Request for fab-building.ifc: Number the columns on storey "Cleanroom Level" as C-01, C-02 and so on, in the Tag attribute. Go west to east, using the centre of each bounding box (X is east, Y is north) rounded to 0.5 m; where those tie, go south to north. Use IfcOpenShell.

First a look at what the model holds.

```python
import ifcopenshell
import ifcopenshell.util.element
import ifcopenshell.util.placement

model = ifcopenshell.open("fab-building.ifc")
print(model.schema)
storey = next(s for s in model.by_type("IfcBuildingStorey") if s.Name == "Cleanroom Level")
columns = [e for e in ifcopenshell.util.element.get_decomposition(storey) if e.is_a("IfcColumn")]
for e in sorted(columns, key=lambda e: e.id()):
    origin = ifcopenshell.util.placement.get_local_placement(e.ObjectPlacement)[:3, 3]
    print(e.id(), e.Tag, e.Name, origin.round(2) + 0.0, sep=" | ")
```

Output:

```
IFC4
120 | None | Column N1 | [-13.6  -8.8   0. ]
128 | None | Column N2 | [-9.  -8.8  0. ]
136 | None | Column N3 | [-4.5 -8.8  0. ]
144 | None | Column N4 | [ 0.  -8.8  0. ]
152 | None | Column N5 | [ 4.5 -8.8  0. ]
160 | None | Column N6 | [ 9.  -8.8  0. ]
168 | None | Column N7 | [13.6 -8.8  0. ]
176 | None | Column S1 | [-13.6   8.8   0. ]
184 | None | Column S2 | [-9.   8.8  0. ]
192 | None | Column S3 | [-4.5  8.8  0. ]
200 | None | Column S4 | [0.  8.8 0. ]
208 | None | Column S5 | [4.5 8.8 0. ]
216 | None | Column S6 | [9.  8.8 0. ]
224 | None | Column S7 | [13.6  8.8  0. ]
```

```python
import ifcopenshell
import ifcopenshell.geom
import ifcopenshell.util.element
import ifcopenshell.util.shape

model = ifcopenshell.open("fab-building.ifc")
settings = ifcopenshell.geom.settings()
settings.set("use-world-coords", True)


def centre(element):
    shape = ifcopenshell.geom.create_shape(settings, element)
    return ifcopenshell.util.shape.get_bbox_centroid(shape.geometry)


storey = next(s for s in model.by_type("IfcBuildingStorey") if s.Name == "Cleanroom Level")
columns = [e for e in ifcopenshell.util.element.get_decomposition(storey) if e.is_a("IfcColumn")]

# Insertion points can sit at a corner or the storey origin, so sort by the geometry (in metres).
centres = {e: centre(e) for e in columns}
columns.sort(key=lambda e: (round(centres[e][0] / 0.5), centres[e][1]))

for i, e in enumerate(columns, start=1):
    number = f"C-{i:02d}"
    e.Tag = number
    print(e.id(), number)

model.write("fab-building-out.ifc")
```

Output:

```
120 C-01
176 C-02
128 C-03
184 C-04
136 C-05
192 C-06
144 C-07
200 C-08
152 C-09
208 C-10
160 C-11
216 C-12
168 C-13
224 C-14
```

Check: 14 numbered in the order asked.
